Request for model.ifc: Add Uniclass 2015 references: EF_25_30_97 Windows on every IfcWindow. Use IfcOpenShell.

First a look at what the model holds.

```python
import ifcopenshell

model = ifcopenshell.open("model.ifc")
print(model.schema)
print("classifications:", [c.Name for c in model.by_type("IfcClassification")])
for ifc_class in ("IfcDoor", "IfcRoof", "IfcStair", "IfcWall", "IfcWindow"):
    print(ifc_class, len(model.by_type(ifc_class)))
```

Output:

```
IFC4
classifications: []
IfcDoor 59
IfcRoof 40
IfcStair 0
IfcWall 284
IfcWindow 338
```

```python
import ifcopenshell
import ifcopenshell.api.classification

model = ifcopenshell.open("model.ifc")

system = ifcopenshell.api.classification.add_classification(model, classification="Uniclass 2015")

codes = {
    "IfcWindow": ("EF_25_30_97", "Windows"),
}
for ifc_class, (code, name) in codes.items():
    products = model.by_type(ifc_class)
    ifcopenshell.api.classification.add_reference(
        model, products=products, classification=system, identification=code, name=name
    )
    print(code, len(products))

model.write("model_v2.ifc")
```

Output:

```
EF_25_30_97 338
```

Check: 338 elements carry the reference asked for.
